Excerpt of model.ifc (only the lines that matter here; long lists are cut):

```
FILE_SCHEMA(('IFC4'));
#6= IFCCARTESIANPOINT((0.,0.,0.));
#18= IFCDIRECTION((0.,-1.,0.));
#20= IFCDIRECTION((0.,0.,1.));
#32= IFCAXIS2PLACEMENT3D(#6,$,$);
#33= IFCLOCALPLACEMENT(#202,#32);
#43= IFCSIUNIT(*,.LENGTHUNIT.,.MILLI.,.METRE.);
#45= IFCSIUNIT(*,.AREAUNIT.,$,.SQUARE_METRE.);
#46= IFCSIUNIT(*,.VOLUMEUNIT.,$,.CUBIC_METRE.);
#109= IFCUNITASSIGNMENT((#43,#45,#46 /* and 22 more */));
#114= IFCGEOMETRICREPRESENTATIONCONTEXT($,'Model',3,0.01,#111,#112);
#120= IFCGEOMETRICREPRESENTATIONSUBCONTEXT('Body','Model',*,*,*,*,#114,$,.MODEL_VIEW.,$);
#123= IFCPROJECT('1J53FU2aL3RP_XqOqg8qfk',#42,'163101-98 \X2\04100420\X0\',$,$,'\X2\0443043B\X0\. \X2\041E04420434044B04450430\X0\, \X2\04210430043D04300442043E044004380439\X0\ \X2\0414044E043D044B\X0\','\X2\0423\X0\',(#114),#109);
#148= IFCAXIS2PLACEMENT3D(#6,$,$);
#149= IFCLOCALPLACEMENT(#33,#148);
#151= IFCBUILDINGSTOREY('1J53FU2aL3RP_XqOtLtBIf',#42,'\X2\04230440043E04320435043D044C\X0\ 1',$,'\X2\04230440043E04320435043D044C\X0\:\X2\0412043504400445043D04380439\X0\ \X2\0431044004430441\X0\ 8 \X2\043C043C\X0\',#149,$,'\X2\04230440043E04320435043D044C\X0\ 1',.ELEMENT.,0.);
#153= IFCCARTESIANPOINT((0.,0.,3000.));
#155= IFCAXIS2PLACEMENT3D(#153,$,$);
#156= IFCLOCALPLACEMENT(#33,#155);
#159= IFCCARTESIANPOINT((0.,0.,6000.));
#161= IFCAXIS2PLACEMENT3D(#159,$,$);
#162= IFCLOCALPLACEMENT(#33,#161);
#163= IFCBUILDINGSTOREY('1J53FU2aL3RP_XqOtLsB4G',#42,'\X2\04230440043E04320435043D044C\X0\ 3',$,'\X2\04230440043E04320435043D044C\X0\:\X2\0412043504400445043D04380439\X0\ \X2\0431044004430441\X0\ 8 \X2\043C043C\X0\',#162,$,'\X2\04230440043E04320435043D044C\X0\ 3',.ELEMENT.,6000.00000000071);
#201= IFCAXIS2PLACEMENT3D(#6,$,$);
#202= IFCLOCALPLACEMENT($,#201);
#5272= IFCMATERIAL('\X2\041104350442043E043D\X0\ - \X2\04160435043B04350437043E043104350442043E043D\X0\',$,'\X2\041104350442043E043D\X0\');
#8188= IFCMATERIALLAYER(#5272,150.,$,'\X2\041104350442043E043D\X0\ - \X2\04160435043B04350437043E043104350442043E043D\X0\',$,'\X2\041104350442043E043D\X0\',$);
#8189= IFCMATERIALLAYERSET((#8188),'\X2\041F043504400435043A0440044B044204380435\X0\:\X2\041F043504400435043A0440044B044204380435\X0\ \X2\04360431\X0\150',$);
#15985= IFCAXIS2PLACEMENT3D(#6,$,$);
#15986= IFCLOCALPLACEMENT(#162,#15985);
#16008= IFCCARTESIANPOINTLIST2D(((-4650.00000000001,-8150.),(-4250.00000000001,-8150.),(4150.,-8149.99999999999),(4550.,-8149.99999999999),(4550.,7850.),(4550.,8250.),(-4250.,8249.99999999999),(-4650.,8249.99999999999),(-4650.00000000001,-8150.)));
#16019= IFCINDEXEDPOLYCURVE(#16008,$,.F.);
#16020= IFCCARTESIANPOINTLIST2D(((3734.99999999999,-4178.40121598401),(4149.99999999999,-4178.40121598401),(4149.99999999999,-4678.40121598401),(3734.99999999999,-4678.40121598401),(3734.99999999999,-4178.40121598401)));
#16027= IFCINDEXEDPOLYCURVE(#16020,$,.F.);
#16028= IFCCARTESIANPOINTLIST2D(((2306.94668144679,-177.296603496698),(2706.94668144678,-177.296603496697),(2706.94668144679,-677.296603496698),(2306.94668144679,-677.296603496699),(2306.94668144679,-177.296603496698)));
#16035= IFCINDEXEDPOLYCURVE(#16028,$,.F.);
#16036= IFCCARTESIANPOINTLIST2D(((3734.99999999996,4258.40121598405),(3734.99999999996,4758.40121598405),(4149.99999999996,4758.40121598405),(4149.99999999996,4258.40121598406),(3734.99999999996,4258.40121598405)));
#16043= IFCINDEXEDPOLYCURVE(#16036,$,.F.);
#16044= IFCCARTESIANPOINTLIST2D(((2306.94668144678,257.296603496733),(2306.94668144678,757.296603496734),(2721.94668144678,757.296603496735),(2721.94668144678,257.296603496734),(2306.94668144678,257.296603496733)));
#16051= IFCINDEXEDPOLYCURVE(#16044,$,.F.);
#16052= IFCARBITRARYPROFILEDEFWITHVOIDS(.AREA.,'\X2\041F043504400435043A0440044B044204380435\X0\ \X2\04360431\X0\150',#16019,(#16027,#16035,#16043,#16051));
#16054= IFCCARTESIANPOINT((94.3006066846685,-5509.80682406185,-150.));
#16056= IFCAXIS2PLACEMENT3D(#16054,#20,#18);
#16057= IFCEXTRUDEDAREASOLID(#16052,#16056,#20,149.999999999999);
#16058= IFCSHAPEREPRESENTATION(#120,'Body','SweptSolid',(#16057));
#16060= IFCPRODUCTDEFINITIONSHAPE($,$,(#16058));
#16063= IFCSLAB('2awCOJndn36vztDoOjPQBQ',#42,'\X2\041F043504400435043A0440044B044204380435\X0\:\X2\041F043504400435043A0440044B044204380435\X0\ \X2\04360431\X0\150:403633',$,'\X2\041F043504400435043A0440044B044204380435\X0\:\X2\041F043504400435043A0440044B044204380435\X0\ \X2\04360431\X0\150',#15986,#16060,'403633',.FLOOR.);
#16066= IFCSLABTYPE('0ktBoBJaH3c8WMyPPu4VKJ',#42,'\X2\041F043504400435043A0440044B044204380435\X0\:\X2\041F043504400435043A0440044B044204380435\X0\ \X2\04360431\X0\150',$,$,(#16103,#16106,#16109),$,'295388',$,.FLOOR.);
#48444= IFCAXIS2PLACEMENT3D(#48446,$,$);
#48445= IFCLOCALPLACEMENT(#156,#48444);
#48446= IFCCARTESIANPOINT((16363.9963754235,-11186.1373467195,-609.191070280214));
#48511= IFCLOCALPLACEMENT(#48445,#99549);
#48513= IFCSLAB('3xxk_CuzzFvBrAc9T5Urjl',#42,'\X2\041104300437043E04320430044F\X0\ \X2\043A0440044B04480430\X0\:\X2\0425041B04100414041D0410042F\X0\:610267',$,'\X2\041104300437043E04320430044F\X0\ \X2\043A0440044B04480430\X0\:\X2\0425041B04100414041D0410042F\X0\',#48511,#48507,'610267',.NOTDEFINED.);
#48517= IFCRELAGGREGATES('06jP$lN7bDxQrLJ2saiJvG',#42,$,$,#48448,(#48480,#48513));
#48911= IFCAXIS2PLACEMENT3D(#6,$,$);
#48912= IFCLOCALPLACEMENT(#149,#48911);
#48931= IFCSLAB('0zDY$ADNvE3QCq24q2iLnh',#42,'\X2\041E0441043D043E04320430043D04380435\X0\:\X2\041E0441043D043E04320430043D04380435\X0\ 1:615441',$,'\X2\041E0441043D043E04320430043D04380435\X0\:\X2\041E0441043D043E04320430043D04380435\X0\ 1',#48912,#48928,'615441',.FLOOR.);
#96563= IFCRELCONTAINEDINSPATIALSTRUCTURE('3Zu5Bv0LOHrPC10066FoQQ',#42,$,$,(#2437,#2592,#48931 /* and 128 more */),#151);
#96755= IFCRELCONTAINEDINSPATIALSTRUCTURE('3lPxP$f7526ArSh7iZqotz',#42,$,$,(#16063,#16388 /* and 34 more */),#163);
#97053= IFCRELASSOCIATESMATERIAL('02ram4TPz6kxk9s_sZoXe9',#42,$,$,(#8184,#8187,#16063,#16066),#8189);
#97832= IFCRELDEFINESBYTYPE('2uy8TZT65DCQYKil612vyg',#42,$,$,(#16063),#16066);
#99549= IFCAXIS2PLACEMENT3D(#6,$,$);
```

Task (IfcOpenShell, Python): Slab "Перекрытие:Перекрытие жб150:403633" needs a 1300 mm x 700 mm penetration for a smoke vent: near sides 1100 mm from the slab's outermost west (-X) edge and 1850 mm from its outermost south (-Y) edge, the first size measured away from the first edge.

```python
import numpy as np
import ifcopenshell
import ifcopenshell.api.feature
import ifcopenshell.api.geometry
import ifcopenshell.api.root
import ifcopenshell.geom
import ifcopenshell.util.placement
import ifcopenshell.util.representation
import ifcopenshell.util.shape
import ifcopenshell.util.unit

model = ifcopenshell.open("model.ifc")
unit_scale = ifcopenshell.util.unit.calculate_unit_scale(model)
settings = ifcopenshell.geom.settings()


def volume(element):
    """Net volume in cubic metres, openings subtracted."""
    shape = ifcopenshell.geom.create_shape(settings, element)
    return ifcopenshell.util.shape.get_volume(shape.geometry)


slab = model.by_guid("2awCOJndn36vztDoOjPQBQ")
before = volume(slab)

# Extent in the slab's own axes, in metres. The edges named are its -X and -Y sides.
slab_shape = ifcopenshell.geom.create_shape(settings, slab)
vertices = ifcopenshell.util.shape.get_vertices(slab_shape.geometry)
x_min, y_min, bottom = vertices.min(axis=0)
top = vertices[:, 2].max()

opening = ifcopenshell.api.root.create_entity(model, ifc_class="IfcOpeningElement", name="Smoke vent opening", predefined_type="OPENING")
context = ifcopenshell.util.representation.get_context(model, "Model", "Body", "MODEL_VIEW")
width, depth = 1.3, 0.7
outline = [(0.0, 0.0), (width, 0.0), (width, depth), (0.0, depth), (0.0, 0.0)]
# Overshoot both faces by 50 mm so the cut is clean.
shape = ifcopenshell.api.geometry.add_slab_representation(
    model, context=context, depth=top - bottom + 0.1, polyline=outline
)
ifcopenshell.api.geometry.assign_representation(model, product=opening, representation=shape)

matrix = ifcopenshell.util.placement.get_local_placement(slab.ObjectPlacement)
matrix[:, 3] = matrix @ np.append(np.array([x_min + 1.1, y_min + 1.85, bottom - 0.05]) / unit_scale, 1.0)
ifcopenshell.api.geometry.edit_object_placement(model, product=opening, matrix=matrix, is_si=False)
ifcopenshell.api.feature.add_feature(model, feature=opening, element=slab)

after = volume(slab)

print(f"slab volume {before:.3f} -> {after:.3f} m3")

model.write("model_updated.ifc")
```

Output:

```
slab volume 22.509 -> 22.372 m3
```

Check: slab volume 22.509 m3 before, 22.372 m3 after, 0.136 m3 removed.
